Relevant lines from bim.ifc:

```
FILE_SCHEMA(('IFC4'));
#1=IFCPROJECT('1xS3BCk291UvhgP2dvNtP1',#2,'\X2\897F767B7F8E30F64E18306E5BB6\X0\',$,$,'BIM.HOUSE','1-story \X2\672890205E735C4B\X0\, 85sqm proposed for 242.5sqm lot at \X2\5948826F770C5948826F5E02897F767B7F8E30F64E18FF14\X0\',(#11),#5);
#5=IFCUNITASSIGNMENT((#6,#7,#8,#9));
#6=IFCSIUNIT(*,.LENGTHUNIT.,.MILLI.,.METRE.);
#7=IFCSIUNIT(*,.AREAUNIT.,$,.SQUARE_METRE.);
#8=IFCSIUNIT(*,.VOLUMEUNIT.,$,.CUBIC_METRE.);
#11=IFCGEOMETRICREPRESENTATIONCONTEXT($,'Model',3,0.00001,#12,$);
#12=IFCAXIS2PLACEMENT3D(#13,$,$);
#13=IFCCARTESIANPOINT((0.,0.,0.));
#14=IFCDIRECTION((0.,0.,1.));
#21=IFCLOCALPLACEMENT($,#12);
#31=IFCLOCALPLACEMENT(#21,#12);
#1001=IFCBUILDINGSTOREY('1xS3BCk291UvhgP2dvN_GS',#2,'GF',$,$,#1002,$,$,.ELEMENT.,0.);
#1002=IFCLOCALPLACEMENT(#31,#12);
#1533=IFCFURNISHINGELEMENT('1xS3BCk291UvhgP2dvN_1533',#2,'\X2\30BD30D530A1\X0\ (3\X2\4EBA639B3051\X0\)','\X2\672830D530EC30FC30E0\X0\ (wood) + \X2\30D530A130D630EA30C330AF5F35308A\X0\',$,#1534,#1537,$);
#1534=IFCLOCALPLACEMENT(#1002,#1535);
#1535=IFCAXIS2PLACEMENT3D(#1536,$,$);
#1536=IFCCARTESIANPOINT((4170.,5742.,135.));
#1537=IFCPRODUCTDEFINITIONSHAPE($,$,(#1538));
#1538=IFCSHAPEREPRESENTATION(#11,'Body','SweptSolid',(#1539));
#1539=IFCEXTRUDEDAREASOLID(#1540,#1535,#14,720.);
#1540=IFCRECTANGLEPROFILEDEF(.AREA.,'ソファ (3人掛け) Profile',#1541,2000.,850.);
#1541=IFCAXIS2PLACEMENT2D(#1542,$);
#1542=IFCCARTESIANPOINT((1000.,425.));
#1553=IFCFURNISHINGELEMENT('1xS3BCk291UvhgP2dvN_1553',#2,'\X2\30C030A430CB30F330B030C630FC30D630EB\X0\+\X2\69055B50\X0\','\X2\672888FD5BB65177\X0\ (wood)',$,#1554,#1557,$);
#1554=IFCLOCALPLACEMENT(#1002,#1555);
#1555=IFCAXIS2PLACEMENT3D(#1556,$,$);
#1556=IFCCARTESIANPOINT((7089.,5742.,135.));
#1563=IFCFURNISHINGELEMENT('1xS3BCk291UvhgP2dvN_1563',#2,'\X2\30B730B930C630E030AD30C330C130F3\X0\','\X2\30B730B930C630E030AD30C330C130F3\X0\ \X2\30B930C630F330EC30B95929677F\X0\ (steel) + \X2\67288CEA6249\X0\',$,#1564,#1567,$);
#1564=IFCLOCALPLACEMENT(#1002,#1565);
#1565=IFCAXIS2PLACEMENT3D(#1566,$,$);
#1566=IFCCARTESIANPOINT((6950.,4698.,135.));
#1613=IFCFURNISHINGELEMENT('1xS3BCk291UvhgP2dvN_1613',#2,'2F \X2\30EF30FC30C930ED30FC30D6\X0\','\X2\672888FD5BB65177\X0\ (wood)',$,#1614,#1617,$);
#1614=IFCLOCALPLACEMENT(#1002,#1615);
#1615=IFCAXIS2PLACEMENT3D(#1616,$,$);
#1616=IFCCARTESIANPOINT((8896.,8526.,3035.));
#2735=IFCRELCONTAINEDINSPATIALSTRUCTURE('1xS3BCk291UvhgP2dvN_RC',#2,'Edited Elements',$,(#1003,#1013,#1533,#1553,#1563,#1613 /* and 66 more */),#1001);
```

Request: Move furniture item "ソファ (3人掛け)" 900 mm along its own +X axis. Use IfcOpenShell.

```python
import ifcopenshell
import ifcopenshell.api.geometry
import ifcopenshell.util.placement
import ifcopenshell.util.unit

model = ifcopenshell.open("bim.ifc")
unit_scale = ifcopenshell.util.unit.calculate_unit_scale(model)

item = model.by_guid("1xS3BCk291UvhgP2dvN_1533")
matrix = ifcopenshell.util.placement.get_local_placement(item.ObjectPlacement)
matrix[:3, 3] += matrix[:3, 0] * 0.9 / unit_scale
ifcopenshell.api.geometry.edit_object_placement(model, product=item, matrix=matrix, is_si=False)

print(ifcopenshell.util.placement.get_local_placement(item.ObjectPlacement).round(3) + 0.0)

model.write("bim_edited.ifc")
```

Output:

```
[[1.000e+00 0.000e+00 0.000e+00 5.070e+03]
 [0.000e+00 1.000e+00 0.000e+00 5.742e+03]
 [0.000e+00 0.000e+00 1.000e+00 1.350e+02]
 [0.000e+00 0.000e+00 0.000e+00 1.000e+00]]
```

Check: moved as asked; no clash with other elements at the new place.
